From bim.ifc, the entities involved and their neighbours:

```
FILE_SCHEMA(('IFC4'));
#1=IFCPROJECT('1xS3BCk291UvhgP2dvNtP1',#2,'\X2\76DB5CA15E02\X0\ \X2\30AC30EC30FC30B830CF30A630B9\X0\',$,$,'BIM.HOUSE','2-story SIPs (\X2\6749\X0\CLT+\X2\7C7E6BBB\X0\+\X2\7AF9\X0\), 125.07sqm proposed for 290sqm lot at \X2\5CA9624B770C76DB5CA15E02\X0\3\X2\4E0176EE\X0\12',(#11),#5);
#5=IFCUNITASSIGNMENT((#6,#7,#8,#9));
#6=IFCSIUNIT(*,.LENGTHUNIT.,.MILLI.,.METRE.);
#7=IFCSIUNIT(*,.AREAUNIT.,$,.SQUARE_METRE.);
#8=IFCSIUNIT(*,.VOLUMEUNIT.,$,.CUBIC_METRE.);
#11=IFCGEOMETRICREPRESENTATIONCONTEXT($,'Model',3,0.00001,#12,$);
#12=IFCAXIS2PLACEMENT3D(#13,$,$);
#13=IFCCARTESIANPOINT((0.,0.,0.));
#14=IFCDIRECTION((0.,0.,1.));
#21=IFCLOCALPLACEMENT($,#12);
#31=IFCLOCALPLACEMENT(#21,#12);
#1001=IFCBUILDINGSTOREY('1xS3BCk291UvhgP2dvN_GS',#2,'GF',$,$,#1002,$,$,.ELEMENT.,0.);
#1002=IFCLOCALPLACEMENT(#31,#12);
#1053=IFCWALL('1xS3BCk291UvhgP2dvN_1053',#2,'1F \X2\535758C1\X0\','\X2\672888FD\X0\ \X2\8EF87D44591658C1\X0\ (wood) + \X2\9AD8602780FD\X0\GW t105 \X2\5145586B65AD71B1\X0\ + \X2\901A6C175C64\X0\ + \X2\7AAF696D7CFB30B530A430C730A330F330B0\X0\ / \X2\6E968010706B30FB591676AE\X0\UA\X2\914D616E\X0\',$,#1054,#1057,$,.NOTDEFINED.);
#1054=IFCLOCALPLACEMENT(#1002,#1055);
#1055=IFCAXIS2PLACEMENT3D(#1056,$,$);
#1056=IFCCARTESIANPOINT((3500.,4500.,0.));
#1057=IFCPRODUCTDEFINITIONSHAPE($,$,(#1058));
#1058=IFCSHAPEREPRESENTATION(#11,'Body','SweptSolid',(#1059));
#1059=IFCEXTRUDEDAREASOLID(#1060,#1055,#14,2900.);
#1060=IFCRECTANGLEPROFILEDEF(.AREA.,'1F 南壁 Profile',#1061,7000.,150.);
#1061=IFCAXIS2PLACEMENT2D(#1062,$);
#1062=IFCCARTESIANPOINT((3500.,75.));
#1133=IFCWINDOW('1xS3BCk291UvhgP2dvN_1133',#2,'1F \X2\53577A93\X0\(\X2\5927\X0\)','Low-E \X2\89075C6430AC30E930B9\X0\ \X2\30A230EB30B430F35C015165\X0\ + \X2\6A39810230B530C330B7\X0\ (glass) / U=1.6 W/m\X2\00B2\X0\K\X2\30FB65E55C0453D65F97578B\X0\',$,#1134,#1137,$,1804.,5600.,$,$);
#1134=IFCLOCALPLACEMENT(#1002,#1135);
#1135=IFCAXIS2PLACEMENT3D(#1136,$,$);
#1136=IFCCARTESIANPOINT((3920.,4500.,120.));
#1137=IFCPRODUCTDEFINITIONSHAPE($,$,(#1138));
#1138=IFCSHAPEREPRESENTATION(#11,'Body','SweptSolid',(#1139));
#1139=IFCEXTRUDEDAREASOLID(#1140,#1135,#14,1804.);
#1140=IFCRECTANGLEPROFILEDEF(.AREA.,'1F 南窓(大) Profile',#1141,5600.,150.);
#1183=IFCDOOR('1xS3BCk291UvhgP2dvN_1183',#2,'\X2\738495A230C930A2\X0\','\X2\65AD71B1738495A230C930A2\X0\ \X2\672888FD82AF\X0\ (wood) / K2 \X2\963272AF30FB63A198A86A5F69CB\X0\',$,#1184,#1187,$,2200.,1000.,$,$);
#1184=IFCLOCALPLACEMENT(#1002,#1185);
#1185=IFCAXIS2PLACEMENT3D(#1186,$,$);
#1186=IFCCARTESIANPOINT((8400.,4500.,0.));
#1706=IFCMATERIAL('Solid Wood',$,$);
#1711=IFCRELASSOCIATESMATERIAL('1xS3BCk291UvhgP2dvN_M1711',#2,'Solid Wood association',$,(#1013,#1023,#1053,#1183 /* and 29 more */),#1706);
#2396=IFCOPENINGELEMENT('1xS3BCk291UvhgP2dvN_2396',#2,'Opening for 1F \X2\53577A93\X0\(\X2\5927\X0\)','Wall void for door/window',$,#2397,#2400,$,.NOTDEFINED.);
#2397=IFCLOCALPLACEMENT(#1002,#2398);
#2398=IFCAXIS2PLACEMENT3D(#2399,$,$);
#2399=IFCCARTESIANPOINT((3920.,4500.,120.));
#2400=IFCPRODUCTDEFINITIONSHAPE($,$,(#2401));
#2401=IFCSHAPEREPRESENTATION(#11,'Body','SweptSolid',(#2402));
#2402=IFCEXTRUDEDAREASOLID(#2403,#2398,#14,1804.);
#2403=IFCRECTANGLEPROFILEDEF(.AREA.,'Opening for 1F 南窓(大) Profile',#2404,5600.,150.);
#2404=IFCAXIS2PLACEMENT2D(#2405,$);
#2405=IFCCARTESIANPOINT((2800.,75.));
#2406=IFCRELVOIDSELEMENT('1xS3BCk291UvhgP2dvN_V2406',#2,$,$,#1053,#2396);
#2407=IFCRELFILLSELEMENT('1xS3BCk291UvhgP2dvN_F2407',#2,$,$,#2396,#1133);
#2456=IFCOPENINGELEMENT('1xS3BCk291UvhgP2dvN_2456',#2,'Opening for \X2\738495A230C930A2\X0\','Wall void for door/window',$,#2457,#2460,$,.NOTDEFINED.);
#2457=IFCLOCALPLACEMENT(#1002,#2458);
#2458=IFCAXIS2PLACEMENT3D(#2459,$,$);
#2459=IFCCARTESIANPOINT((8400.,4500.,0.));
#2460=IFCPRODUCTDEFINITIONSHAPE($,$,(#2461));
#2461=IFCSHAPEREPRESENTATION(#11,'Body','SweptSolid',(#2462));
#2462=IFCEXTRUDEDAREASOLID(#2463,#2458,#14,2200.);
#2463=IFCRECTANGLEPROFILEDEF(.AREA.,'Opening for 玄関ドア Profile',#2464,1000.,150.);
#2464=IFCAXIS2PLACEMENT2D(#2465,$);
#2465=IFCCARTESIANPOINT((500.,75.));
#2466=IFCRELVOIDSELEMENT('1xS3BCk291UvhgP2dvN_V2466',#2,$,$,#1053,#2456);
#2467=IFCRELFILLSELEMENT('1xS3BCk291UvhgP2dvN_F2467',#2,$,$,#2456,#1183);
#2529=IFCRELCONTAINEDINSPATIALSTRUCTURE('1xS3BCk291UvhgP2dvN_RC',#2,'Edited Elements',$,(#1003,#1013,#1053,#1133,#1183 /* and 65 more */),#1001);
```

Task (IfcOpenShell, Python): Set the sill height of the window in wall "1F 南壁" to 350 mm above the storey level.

```python
import numpy as np
import ifcopenshell
import ifcopenshell.api.geometry
import ifcopenshell.geom
import ifcopenshell.util.element
import ifcopenshell.util.placement
import ifcopenshell.util.shape
import ifcopenshell.util.unit

model = ifcopenshell.open("bim.ifc")
unit_scale = ifcopenshell.util.unit.calculate_unit_scale(model)

window = model.by_id(1133)
opening = window.FillsVoids[0].RelatingOpeningElement
storey = ifcopenshell.util.element.get_container(window, ifc_class="IfcBuildingStorey")
level = ifcopenshell.util.placement.get_local_placement(storey.ObjectPlacement)[2, 3]

# The opening's origin need not be at the sill, so measure its lowest point.
shape = ifcopenshell.geom.create_shape(ifcopenshell.geom.settings(), opening)
bottom = ifcopenshell.util.shape.get_shape_bottom_elevation(shape, shape.geometry) / unit_scale
dz = level + 350.0 - bottom

shift = np.array([0.0, 0.0, dz])
# The window is not placed relative to its opening, so move both.
for product in (opening, window):
    matrix = ifcopenshell.util.placement.get_local_placement(product.ObjectPlacement)
    matrix[:3, 3] += shift
    ifcopenshell.api.geometry.edit_object_placement(model, product=product, matrix=matrix, is_si=False)

print(f"moved by {dz * unit_scale:+.3f} m")

model.write("bim-out.ifc")
```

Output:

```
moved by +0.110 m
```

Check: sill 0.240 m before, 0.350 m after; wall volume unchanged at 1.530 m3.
